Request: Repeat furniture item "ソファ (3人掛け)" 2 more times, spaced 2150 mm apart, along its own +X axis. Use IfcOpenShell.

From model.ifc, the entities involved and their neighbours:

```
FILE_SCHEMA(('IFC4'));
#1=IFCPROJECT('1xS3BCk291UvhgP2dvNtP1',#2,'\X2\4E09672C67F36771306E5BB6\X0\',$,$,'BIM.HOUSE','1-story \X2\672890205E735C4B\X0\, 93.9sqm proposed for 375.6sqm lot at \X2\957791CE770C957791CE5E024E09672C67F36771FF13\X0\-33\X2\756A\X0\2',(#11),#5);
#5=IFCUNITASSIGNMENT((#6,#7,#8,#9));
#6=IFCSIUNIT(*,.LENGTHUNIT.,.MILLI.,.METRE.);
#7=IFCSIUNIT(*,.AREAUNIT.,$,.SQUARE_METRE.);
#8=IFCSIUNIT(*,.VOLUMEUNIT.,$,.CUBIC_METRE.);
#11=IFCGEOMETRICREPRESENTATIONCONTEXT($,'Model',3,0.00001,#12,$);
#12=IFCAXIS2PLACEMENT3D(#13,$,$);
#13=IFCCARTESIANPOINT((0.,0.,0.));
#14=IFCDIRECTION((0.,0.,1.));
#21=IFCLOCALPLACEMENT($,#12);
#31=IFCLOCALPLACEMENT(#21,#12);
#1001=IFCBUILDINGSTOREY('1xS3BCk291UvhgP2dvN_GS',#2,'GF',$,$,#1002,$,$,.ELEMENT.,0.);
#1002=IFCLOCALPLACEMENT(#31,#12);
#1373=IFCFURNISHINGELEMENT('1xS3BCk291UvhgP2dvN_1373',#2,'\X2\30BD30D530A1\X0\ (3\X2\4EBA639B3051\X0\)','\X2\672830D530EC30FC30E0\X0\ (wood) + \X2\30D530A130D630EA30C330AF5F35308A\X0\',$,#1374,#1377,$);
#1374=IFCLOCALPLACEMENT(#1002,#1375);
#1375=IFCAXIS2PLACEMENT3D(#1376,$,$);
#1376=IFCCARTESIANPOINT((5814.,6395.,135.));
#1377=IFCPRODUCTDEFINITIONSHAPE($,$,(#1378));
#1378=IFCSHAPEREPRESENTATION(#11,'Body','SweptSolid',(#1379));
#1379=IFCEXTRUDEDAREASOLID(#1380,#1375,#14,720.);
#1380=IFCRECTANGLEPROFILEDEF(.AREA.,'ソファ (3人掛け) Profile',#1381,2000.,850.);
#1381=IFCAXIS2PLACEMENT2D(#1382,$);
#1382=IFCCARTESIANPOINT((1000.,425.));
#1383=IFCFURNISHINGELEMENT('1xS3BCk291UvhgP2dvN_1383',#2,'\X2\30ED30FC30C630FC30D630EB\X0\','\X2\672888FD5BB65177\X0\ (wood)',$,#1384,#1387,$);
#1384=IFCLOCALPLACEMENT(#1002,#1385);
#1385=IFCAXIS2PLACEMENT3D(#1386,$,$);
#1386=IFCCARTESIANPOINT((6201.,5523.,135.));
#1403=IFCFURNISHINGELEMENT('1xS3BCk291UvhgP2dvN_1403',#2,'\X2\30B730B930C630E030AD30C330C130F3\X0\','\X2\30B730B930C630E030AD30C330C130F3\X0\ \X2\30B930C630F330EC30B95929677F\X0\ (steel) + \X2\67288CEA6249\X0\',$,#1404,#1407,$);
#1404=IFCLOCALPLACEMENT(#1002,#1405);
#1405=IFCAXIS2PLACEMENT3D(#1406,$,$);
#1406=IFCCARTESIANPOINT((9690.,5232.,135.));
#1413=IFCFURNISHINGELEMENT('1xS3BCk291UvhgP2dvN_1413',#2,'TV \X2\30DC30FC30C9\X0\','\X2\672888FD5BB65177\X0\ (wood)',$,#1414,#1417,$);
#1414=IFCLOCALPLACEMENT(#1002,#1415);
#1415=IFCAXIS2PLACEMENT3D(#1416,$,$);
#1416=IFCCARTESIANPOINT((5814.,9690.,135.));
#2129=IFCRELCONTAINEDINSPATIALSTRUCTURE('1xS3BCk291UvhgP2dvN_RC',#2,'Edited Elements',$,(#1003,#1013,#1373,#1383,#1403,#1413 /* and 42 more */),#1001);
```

```python
import ifcopenshell
import ifcopenshell.api.geometry
import ifcopenshell.api.root
import ifcopenshell.util.element
import ifcopenshell.util.placement
import ifcopenshell.util.unit

model = ifcopenshell.open("model.ifc")
unit_scale = ifcopenshell.util.unit.calculate_unit_scale(model)


def reuse_history(source, copy):
    """copy_class also copies each property set's owner history, people and application; keep the originals."""
    for rel in copy.IsDefinedBy:
        if rel.is_a("IfcRelDefinesByProperties") and (history := rel.RelatingPropertyDefinition.OwnerHistory):
            rel.RelatingPropertyDefinition.OwnerHistory = source.OwnerHistory
            ifcopenshell.util.element.remove_deep2(model, history)


source = model.by_guid("1xS3BCk291UvhgP2dvN_1373")
base = ifcopenshell.util.placement.get_local_placement(source.ObjectPlacement)
step = base[:3, 0] * 2.15 / unit_scale

for i in range(1, 3):
    copy = ifcopenshell.api.root.copy_class(model, product=source)
    copy.Representation = ifcopenshell.util.element.copy_deep(
        model, source.Representation, exclude=["IfcGeometricRepresentationContext", "IfcRepresentationMap"]
    )
    reuse_history(source, copy)
    matrix = base.copy()
    matrix[:3, 3] += i * step
    print("added at", matrix[:3, 3].round(3) + 0.0)
    ifcopenshell.api.geometry.edit_object_placement(model, product=copy, matrix=matrix, is_si=False)

model.write("model_updated.ifc")
```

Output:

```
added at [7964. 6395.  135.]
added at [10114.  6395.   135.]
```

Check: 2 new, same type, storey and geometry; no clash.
